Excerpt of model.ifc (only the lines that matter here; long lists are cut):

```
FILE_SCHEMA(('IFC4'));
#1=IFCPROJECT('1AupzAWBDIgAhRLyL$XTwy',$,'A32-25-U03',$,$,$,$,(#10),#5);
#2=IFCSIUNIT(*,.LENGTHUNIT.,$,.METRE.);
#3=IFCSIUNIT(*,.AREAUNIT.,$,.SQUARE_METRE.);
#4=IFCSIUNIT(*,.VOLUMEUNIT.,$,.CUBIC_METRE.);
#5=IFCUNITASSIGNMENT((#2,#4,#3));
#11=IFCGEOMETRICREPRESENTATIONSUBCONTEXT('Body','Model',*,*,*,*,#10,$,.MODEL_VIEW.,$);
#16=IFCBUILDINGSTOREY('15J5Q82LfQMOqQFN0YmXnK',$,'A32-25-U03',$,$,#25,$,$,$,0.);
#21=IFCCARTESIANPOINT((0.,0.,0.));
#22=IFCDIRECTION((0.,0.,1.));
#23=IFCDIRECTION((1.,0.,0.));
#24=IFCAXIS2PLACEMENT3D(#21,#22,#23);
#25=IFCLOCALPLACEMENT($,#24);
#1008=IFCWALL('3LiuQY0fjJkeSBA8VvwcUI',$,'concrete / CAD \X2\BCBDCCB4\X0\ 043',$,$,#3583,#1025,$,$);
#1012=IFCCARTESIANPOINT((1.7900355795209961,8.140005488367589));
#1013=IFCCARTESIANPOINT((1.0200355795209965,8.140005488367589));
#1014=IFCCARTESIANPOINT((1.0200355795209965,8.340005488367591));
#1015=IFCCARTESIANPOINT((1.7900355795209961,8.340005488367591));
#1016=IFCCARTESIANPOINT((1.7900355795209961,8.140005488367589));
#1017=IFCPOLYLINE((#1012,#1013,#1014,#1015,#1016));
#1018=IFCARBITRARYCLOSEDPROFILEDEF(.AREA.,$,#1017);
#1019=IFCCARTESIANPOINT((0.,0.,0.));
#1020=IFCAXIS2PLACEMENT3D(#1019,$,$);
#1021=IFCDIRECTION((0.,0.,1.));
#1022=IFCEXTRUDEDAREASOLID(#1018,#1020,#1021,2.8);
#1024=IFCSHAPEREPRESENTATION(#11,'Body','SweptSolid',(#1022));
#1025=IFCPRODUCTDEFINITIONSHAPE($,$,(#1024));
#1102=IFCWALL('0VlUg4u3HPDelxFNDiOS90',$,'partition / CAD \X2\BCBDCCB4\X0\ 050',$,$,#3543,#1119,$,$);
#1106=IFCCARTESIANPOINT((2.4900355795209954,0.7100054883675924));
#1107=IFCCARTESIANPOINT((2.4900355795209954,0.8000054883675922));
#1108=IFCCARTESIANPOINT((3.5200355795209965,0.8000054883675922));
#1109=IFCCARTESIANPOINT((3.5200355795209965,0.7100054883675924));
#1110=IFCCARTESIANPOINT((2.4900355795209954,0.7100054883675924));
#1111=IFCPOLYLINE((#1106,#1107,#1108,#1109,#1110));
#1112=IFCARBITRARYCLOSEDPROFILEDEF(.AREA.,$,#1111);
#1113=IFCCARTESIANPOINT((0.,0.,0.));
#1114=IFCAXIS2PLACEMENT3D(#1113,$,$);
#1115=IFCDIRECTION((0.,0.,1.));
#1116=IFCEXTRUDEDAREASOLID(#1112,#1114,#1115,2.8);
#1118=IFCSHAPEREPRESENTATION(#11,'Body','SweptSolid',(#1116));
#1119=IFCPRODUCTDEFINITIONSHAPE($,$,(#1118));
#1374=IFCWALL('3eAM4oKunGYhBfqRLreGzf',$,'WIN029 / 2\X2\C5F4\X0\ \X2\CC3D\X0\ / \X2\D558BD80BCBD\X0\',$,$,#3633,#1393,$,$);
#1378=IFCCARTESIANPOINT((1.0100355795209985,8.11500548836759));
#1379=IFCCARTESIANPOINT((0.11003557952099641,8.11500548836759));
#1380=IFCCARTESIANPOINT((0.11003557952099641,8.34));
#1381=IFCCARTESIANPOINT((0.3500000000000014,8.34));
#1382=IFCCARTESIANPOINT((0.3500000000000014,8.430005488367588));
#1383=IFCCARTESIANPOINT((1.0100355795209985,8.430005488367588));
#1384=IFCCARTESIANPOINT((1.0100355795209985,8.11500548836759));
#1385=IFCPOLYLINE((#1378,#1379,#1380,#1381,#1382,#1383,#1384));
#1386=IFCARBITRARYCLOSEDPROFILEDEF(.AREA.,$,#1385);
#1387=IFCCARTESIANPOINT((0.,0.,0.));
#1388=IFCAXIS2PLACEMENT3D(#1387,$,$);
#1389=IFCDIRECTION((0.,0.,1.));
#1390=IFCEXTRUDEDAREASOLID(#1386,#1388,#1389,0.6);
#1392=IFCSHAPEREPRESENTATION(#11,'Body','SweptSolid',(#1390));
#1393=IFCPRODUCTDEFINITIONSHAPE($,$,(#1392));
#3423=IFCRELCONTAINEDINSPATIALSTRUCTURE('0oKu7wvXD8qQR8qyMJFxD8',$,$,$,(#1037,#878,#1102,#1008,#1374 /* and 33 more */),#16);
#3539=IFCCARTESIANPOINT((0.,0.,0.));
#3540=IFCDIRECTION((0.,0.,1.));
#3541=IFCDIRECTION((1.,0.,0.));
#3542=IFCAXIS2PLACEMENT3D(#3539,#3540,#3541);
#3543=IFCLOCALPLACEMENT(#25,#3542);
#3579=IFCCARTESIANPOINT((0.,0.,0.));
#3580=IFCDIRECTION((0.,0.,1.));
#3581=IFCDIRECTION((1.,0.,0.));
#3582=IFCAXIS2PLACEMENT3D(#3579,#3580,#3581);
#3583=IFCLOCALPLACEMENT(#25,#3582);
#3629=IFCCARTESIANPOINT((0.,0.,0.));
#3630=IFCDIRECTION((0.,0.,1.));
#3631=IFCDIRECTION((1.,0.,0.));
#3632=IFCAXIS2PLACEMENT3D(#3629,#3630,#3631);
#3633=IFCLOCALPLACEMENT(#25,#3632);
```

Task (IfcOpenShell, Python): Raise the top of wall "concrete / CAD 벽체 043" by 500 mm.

```python
import ifcopenshell
import ifcopenshell.geom
import ifcopenshell.util.representation
import ifcopenshell.util.shape
import ifcopenshell.util.unit

model = ifcopenshell.open("model.ifc")
unit_scale = ifcopenshell.util.unit.calculate_unit_scale(model)
settings = ifcopenshell.geom.settings()


def volume(element):
    """Net volume in cubic metres, openings subtracted."""
    shape = ifcopenshell.geom.create_shape(settings, element)
    return ifcopenshell.util.shape.get_volume(shape.geometry)


wall = model.by_id(1008)
before = volume(wall)

body = ifcopenshell.util.representation.get_representation(wall, "Model", "Body")
solid = body.Items[0]
old_height = solid.Depth
solid.Depth += 0.5 / unit_scale
after = volume(wall)

print(f"height {old_height:g} -> {solid.Depth:g}, volume {before:.3f} -> {after:.3f} m3")

model.write("model_edited.ifc")
```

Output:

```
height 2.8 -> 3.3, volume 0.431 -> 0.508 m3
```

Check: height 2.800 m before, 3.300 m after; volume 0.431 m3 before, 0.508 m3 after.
